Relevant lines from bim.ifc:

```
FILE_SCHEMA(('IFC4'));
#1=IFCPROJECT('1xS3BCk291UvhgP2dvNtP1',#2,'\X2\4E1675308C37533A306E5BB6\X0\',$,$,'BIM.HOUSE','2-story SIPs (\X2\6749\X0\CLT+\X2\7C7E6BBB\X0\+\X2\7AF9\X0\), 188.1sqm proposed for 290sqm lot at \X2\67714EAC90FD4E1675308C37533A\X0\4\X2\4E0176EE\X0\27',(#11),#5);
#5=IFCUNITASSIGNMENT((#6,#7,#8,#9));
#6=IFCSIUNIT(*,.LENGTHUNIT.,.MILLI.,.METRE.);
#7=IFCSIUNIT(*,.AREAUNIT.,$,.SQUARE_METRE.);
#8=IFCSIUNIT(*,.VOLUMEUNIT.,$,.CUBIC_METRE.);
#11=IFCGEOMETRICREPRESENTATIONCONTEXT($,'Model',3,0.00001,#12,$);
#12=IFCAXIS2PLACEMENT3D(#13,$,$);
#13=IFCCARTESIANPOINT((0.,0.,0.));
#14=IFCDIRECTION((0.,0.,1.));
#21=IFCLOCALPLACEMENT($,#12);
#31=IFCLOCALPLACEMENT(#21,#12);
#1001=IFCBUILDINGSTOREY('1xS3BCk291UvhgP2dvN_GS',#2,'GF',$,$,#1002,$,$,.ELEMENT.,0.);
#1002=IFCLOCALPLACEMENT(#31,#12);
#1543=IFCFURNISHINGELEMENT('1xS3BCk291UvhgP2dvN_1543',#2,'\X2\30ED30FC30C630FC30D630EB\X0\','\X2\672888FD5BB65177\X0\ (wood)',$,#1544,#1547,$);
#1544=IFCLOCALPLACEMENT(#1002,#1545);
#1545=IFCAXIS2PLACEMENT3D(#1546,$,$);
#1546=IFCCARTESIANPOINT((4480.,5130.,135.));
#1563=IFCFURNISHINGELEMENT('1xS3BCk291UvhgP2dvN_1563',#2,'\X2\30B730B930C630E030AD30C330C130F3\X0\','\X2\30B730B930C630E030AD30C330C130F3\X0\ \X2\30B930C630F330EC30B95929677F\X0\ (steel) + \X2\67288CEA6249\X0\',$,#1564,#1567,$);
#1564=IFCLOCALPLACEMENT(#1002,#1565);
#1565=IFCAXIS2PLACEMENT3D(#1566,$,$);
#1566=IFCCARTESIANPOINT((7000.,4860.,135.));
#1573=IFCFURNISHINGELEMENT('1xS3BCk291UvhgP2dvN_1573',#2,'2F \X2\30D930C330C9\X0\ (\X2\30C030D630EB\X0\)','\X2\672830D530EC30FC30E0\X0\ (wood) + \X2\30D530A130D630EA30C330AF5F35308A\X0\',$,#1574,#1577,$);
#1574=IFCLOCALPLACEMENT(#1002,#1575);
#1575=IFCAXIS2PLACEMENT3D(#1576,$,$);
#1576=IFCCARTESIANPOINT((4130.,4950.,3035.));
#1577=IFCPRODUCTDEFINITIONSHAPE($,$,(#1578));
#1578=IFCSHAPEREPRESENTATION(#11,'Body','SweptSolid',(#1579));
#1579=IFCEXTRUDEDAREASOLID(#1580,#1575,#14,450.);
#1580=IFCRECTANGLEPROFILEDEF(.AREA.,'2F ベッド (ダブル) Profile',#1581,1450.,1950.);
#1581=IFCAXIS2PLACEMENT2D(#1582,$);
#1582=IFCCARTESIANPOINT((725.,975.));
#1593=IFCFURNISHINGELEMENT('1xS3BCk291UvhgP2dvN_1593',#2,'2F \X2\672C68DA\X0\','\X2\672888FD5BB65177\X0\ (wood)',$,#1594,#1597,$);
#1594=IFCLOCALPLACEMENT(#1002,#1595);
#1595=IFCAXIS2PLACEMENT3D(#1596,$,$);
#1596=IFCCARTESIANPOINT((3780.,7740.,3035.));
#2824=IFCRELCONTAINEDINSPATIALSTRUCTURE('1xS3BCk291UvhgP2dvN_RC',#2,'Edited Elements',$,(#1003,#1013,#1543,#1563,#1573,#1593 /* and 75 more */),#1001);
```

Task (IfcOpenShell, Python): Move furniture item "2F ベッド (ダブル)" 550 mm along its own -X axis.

```python
import ifcopenshell
import ifcopenshell.api.geometry
import ifcopenshell.util.placement
import ifcopenshell.util.unit

model = ifcopenshell.open("bim.ifc")
unit_scale = ifcopenshell.util.unit.calculate_unit_scale(model)

item = model.by_guid("1xS3BCk291UvhgP2dvN_1573")
matrix = ifcopenshell.util.placement.get_local_placement(item.ObjectPlacement)
matrix[:3, 3] -= matrix[:3, 0] * 0.55 / unit_scale
ifcopenshell.api.geometry.edit_object_placement(model, product=item, matrix=matrix, is_si=False)

print(ifcopenshell.util.placement.get_local_placement(item.ObjectPlacement).round(3) + 0.0)

model.write("bim_updated.ifc")
```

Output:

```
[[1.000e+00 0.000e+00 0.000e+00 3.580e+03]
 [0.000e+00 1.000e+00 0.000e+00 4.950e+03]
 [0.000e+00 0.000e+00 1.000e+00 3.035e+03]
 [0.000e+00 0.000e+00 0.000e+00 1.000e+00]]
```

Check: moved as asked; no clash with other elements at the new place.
